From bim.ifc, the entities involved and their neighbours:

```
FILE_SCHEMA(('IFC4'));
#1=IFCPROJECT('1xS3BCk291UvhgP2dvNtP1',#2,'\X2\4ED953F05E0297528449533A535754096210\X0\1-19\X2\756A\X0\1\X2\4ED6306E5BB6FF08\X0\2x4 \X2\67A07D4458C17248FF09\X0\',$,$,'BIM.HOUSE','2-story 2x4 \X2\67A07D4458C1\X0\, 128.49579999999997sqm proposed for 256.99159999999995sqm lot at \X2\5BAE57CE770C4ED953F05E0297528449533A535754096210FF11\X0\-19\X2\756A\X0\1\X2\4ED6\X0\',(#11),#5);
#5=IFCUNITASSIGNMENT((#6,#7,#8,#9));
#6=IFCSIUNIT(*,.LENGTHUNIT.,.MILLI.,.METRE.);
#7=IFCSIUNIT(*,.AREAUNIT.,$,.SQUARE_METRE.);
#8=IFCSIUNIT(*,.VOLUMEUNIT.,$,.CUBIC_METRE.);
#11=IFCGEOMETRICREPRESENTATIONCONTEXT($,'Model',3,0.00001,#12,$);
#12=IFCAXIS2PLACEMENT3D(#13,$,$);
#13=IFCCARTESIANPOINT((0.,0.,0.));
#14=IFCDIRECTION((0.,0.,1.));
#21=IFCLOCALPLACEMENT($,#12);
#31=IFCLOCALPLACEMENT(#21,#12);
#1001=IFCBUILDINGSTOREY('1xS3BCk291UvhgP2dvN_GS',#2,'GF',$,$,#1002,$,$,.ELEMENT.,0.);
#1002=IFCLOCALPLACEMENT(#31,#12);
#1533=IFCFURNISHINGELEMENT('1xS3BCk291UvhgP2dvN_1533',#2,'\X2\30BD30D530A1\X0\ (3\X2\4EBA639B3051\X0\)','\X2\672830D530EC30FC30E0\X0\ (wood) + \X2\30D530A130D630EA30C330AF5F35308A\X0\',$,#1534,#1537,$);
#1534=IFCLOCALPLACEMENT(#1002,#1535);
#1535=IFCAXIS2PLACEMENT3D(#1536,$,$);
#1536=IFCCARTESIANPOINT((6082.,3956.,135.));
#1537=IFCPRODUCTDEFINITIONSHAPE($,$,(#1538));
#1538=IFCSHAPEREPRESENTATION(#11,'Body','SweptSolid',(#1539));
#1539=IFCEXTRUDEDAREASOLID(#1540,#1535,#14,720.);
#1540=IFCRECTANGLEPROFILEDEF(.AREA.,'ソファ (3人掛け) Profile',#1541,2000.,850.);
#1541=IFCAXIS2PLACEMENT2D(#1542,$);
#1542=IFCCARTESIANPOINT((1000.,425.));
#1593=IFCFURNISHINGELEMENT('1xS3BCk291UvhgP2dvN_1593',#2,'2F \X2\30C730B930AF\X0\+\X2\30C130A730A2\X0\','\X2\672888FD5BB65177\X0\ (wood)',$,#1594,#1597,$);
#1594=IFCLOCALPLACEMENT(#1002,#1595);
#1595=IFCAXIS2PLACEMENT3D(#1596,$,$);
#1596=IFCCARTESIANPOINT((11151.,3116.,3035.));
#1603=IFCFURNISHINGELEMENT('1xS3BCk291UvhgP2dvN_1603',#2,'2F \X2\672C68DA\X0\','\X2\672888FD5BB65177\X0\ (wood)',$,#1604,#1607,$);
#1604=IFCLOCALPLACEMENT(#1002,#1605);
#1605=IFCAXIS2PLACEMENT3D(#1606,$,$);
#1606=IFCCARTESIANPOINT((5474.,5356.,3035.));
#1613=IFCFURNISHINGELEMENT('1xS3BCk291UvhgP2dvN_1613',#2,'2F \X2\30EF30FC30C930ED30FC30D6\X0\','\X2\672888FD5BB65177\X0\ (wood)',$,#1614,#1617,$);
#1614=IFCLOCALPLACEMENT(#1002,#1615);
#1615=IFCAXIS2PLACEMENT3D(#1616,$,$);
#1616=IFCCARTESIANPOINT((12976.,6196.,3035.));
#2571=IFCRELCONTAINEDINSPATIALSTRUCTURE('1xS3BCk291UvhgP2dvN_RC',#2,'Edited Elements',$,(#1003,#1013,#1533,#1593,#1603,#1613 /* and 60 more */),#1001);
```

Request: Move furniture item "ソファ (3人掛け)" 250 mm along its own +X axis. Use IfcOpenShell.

```python
import ifcopenshell
import ifcopenshell.api.geometry
import ifcopenshell.util.placement

model = ifcopenshell.open("bim.ifc")

item = model.by_guid("1xS3BCk291UvhgP2dvN_1533")
matrix = ifcopenshell.util.placement.get_local_placement(item.ObjectPlacement)
matrix[:3, 3] += matrix[:3, 0] * 250.0
ifcopenshell.api.geometry.edit_object_placement(model, product=item, matrix=matrix, is_si=False)

print(ifcopenshell.util.placement.get_local_placement(item.ObjectPlacement).round(3) + 0.0)

model.write("bim_v2.ifc")
```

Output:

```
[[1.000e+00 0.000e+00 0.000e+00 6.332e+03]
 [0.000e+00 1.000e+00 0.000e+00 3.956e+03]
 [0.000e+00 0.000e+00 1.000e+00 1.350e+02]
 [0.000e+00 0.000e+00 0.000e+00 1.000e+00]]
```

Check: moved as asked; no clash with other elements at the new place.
